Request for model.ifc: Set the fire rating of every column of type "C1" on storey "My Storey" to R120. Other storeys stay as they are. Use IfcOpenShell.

First a look at what the model holds.

```python
import ifcopenshell
import ifcopenshell.util.element

model = ifcopenshell.open("model.ifc")
print(model.schema)
storey = next(s for s in model.by_type("IfcBuildingStorey") if s.Name == "My Storey")
columns = [e for e in ifcopenshell.util.element.get_decomposition(storey) if e.is_a("IfcColumn")]
seen = {}
for e in columns:
    element_type = ifcopenshell.util.element.get_type(e)
    key = (element_type.Name if element_type != e and element_type else None, ifcopenshell.util.element.get_pset(e, "Pset_ColumnCommon", "FireRating"))
    seen[key] = seen.get(key, 0) + 1
for (name, value), count in sorted(seen.items(), key=str):
    print(count, "x", name, "|", value)
```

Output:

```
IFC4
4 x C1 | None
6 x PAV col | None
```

```python
import ifcopenshell
import ifcopenshell.api.pset
import ifcopenshell.util.element

model = ifcopenshell.open("model.ifc")

storey = next(s for s in model.by_type("IfcBuildingStorey") if s.Name == "My Storey")
columns = [e for e in ifcopenshell.util.element.get_decomposition(storey) if e.is_a("IfcColumn")]

count = 0
for e in columns:
    element_type = ifcopenshell.util.element.get_type(e)
    if element_type in (None, e) or element_type.Name != "C1":
        continue
    # add_pset returns the element's existing set when there is one.
    pset = ifcopenshell.api.pset.add_pset(model, product=e, name="Pset_ColumnCommon")
    ifcopenshell.api.pset.edit_pset(model, pset=pset, properties={"FireRating": "R120"})
    count += 1

print(count, "columns updated")

model.write("model_updated.ifc")
```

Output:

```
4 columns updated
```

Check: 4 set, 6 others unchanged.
